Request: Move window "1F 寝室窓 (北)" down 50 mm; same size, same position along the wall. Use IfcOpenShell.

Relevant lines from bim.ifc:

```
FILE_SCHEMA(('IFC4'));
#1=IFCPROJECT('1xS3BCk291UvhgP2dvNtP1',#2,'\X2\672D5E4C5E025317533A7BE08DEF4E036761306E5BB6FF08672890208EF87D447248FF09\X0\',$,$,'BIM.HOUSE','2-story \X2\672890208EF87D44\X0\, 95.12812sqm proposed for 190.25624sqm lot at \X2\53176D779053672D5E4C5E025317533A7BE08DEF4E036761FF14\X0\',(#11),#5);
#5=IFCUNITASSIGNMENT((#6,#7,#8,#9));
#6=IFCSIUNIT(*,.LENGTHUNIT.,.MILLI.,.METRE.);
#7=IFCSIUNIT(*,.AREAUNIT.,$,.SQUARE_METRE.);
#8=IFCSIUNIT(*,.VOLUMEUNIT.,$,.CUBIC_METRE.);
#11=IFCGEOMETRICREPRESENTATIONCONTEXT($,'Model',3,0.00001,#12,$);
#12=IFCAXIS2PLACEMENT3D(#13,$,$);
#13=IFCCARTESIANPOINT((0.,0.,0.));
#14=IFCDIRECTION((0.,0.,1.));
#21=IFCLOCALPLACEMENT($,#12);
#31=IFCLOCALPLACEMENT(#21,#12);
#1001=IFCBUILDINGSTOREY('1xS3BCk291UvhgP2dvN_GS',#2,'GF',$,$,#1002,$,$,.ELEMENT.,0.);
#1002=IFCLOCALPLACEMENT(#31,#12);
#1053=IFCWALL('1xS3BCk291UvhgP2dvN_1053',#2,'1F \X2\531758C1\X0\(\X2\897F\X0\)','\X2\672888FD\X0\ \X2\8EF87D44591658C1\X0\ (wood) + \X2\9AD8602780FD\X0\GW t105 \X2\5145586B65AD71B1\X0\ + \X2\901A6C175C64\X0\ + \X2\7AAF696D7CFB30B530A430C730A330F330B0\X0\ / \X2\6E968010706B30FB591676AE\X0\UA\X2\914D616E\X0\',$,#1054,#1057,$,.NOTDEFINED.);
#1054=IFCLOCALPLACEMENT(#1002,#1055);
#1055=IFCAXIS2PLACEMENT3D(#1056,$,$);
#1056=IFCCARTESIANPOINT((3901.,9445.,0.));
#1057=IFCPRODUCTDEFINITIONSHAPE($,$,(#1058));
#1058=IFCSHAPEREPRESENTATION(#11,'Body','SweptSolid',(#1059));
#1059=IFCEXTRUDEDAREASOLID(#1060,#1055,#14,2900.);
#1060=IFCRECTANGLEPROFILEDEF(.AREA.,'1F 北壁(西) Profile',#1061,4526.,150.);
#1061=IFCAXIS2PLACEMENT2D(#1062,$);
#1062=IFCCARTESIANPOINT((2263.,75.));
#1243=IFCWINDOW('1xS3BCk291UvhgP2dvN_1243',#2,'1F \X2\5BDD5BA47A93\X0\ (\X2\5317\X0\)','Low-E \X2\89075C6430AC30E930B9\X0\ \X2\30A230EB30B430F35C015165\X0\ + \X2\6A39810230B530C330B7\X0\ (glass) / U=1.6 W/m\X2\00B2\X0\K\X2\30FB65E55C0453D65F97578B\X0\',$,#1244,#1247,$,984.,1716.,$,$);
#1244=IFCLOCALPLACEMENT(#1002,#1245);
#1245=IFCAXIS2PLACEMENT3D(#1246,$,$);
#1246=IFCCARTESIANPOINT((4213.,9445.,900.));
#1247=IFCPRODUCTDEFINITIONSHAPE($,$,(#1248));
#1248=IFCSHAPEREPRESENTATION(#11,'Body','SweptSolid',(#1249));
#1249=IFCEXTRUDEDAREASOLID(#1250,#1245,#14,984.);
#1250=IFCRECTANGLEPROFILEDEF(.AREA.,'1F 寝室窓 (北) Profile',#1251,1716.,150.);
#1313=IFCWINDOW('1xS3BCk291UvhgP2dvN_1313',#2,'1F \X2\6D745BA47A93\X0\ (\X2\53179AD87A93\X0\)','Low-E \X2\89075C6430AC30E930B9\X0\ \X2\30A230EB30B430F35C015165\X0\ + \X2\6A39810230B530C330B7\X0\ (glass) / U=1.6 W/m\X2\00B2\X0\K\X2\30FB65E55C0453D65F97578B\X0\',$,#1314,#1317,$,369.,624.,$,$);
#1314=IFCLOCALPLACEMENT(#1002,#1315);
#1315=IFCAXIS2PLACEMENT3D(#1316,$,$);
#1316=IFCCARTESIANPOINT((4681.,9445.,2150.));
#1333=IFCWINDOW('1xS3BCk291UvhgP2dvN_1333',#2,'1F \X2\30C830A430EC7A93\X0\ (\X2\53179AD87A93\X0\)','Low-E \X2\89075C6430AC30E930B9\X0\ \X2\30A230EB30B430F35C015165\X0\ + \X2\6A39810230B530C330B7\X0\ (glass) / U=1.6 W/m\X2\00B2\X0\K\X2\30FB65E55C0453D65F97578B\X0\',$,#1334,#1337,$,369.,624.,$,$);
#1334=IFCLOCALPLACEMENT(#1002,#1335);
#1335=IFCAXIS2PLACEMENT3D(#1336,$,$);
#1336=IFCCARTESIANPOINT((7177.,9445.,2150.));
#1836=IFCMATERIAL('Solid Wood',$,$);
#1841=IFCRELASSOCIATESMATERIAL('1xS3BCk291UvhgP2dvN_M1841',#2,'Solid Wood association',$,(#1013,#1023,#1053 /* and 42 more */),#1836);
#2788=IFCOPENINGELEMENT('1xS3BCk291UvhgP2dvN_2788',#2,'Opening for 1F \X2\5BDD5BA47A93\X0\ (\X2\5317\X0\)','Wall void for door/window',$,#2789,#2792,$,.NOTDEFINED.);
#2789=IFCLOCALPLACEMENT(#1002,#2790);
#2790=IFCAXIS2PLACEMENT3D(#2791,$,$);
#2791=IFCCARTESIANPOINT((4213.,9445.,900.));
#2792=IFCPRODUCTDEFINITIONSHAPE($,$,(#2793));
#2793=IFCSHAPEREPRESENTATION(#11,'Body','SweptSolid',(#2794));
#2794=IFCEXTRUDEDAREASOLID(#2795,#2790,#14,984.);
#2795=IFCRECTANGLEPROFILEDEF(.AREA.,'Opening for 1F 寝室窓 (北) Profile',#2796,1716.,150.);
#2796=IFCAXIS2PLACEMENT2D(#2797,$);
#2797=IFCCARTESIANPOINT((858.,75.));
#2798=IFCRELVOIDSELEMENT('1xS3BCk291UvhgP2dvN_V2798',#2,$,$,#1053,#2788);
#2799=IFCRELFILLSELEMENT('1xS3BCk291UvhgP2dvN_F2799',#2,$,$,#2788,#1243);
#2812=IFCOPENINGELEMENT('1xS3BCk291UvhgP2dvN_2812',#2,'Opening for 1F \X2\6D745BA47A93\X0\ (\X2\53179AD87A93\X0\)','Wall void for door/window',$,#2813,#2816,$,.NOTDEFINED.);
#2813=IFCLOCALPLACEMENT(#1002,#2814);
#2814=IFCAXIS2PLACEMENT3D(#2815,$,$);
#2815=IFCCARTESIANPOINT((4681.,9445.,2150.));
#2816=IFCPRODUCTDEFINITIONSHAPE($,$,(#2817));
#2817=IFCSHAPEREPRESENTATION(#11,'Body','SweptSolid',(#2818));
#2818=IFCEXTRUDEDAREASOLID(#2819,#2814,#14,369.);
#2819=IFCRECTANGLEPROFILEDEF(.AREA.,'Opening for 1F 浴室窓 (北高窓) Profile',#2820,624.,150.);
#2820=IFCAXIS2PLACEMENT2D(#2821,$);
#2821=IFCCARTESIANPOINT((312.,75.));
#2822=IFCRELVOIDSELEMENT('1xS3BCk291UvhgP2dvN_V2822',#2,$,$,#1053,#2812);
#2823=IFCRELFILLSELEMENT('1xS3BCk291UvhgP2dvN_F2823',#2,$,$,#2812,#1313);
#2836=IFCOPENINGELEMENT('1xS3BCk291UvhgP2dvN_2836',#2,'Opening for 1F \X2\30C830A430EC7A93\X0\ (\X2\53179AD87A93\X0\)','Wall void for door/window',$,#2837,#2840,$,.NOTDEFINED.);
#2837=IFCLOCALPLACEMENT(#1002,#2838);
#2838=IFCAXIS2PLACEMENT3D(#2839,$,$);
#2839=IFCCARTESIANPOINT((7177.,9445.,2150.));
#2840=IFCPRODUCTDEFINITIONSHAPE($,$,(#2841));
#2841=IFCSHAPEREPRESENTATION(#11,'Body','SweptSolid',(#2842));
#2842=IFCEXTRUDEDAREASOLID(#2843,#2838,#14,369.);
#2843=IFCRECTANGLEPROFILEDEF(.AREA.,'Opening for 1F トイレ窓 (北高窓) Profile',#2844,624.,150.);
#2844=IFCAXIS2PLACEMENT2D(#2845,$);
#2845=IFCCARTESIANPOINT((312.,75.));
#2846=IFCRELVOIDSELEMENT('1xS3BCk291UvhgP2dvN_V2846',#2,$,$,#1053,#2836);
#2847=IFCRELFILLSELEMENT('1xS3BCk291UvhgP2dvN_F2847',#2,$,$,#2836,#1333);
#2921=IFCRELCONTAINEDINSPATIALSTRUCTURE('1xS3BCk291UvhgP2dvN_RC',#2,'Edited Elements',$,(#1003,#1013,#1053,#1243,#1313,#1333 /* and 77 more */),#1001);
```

```python
import numpy as np
import ifcopenshell
import ifcopenshell.api.geometry
import ifcopenshell.util.placement
import ifcopenshell.util.unit

model = ifcopenshell.open("bim.ifc")
unit_scale = ifcopenshell.util.unit.calculate_unit_scale(model)

window = model.by_id(1243)
opening = window.FillsVoids[0].RelatingOpeningElement
dz = -0.05 / unit_scale

shift = np.array([0.0, 0.0, dz])
# The window is not placed relative to its opening, so move both.
for product in (opening, window):
    matrix = ifcopenshell.util.placement.get_local_placement(product.ObjectPlacement)
    matrix[:3, 3] += shift
    ifcopenshell.api.geometry.edit_object_placement(model, product=product, matrix=matrix, is_si=False)

print(f"moved by {dz * unit_scale:+.3f} m")

model.write("bim_edited.ifc")
```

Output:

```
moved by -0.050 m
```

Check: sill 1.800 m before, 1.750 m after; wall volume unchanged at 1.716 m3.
